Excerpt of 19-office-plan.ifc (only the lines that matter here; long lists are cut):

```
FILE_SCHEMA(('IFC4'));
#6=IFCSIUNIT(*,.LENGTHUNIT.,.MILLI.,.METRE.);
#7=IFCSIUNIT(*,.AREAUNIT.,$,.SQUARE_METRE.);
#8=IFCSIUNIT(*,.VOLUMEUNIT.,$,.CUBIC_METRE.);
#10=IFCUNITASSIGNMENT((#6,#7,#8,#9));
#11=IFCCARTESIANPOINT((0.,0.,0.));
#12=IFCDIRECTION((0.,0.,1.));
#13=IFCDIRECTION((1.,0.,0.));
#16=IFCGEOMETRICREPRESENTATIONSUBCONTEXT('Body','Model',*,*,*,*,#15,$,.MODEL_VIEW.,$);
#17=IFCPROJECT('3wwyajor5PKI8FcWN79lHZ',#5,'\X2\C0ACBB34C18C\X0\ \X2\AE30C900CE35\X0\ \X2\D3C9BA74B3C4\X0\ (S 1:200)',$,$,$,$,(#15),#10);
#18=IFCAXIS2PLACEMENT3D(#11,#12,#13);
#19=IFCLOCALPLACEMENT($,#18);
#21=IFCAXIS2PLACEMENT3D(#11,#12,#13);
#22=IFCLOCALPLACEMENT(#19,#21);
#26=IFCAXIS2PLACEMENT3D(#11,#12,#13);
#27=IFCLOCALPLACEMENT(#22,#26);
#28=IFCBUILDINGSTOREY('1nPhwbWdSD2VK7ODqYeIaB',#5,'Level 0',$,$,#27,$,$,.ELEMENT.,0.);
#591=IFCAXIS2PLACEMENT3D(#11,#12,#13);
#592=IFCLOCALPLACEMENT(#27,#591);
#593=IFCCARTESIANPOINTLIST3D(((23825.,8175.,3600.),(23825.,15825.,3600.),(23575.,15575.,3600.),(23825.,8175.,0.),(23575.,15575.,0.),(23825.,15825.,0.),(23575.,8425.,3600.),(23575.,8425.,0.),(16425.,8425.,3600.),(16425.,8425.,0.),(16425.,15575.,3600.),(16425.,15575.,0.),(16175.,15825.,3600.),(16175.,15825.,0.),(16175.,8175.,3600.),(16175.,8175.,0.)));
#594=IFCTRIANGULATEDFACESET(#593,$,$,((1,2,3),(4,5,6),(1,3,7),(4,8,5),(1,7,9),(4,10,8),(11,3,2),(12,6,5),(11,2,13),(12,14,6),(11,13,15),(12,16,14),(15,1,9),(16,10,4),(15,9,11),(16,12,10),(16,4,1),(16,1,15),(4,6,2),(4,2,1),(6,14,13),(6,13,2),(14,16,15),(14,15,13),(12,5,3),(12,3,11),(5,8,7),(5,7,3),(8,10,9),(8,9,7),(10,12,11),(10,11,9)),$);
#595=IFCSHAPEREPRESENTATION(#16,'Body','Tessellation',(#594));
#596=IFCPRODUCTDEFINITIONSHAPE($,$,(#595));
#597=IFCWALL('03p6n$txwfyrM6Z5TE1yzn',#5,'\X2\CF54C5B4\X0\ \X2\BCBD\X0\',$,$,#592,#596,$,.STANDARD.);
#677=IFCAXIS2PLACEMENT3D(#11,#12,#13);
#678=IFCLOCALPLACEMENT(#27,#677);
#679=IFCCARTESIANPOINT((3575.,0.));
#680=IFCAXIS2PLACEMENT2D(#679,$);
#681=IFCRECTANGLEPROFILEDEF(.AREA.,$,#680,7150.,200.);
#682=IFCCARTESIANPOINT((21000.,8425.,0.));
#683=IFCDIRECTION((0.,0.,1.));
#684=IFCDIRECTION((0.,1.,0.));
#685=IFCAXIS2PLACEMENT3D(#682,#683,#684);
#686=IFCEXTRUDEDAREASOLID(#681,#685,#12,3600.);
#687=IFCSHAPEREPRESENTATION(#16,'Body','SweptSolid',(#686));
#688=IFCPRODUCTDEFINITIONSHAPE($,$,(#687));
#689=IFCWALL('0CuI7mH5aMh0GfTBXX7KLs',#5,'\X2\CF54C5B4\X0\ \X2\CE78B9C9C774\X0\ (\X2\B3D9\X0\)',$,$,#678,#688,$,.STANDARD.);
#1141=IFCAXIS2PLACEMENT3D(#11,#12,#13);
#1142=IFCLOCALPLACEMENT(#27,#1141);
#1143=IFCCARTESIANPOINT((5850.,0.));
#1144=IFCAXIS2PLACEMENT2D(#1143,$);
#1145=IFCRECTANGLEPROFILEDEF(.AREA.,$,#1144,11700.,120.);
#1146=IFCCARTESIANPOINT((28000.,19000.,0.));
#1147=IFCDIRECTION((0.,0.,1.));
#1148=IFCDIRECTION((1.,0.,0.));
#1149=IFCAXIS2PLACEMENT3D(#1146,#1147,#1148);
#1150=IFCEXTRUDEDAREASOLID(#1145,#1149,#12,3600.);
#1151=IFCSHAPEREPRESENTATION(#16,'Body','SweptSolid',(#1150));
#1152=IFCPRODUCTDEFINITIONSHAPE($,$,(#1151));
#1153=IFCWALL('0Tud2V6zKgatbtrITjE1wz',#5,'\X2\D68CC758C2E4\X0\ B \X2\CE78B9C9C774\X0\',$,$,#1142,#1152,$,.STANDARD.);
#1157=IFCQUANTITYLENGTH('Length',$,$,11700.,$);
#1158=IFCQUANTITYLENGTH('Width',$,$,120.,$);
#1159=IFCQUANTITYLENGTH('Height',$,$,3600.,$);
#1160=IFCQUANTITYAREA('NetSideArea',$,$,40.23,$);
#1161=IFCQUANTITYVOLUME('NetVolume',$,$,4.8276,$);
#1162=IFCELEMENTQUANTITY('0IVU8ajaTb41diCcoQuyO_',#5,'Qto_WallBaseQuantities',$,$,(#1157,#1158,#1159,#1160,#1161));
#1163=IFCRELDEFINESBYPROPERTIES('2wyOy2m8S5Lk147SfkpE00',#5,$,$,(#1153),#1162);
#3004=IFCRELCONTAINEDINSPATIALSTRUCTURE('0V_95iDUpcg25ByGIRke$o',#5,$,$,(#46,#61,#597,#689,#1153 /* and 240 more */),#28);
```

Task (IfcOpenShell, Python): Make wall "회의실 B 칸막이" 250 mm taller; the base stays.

```python
import ifcopenshell
import ifcopenshell.api.pset
import ifcopenshell.geom
import ifcopenshell.util.element
import ifcopenshell.util.representation
import ifcopenshell.util.shape
import ifcopenshell.util.unit

model = ifcopenshell.open("19-office-plan.ifc")
unit_scale = ifcopenshell.util.unit.calculate_unit_scale(model)
area_scale = ifcopenshell.util.unit.calculate_unit_scale(model, "AREAUNIT")
volume_scale = ifcopenshell.util.unit.calculate_unit_scale(model, "VOLUMEUNIT")
settings = ifcopenshell.geom.settings()


def volume(element):
    """Net volume in cubic metres, openings subtracted."""
    shape = ifcopenshell.geom.create_shape(settings, element)
    return ifcopenshell.util.shape.get_volume(shape.geometry)


wall = model.by_guid("0Tud2V6zKgatbtrITjE1wz")
before = volume(wall)

body = ifcopenshell.util.representation.get_representation(wall, "Model", "Body")
solid = body.Items[0]
old_height = solid.Depth
solid.Depth += 0.25 / unit_scale
after = volume(wall)
thickness = 0.12  # wall thickness in metres

# Update the stored height, areas and volumes.
qto = model.by_id(ifcopenshell.util.element.get_pset(wall, "Qto_WallBaseQuantities", should_inherit=False)["id"])
ifcopenshell.api.pset.edit_qto(model, qto=qto, properties={
    "Height": solid.Depth,
    "NetSideArea": after / thickness / area_scale,
    "NetVolume": after / volume_scale,
})

print(f"height {old_height:g} -> {solid.Depth:g}, volume {before:.3f} -> {after:.3f} m3")

model.write("19-office-plan-out.ifc")
```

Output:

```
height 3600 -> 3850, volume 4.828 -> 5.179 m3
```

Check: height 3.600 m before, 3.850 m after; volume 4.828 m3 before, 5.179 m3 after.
